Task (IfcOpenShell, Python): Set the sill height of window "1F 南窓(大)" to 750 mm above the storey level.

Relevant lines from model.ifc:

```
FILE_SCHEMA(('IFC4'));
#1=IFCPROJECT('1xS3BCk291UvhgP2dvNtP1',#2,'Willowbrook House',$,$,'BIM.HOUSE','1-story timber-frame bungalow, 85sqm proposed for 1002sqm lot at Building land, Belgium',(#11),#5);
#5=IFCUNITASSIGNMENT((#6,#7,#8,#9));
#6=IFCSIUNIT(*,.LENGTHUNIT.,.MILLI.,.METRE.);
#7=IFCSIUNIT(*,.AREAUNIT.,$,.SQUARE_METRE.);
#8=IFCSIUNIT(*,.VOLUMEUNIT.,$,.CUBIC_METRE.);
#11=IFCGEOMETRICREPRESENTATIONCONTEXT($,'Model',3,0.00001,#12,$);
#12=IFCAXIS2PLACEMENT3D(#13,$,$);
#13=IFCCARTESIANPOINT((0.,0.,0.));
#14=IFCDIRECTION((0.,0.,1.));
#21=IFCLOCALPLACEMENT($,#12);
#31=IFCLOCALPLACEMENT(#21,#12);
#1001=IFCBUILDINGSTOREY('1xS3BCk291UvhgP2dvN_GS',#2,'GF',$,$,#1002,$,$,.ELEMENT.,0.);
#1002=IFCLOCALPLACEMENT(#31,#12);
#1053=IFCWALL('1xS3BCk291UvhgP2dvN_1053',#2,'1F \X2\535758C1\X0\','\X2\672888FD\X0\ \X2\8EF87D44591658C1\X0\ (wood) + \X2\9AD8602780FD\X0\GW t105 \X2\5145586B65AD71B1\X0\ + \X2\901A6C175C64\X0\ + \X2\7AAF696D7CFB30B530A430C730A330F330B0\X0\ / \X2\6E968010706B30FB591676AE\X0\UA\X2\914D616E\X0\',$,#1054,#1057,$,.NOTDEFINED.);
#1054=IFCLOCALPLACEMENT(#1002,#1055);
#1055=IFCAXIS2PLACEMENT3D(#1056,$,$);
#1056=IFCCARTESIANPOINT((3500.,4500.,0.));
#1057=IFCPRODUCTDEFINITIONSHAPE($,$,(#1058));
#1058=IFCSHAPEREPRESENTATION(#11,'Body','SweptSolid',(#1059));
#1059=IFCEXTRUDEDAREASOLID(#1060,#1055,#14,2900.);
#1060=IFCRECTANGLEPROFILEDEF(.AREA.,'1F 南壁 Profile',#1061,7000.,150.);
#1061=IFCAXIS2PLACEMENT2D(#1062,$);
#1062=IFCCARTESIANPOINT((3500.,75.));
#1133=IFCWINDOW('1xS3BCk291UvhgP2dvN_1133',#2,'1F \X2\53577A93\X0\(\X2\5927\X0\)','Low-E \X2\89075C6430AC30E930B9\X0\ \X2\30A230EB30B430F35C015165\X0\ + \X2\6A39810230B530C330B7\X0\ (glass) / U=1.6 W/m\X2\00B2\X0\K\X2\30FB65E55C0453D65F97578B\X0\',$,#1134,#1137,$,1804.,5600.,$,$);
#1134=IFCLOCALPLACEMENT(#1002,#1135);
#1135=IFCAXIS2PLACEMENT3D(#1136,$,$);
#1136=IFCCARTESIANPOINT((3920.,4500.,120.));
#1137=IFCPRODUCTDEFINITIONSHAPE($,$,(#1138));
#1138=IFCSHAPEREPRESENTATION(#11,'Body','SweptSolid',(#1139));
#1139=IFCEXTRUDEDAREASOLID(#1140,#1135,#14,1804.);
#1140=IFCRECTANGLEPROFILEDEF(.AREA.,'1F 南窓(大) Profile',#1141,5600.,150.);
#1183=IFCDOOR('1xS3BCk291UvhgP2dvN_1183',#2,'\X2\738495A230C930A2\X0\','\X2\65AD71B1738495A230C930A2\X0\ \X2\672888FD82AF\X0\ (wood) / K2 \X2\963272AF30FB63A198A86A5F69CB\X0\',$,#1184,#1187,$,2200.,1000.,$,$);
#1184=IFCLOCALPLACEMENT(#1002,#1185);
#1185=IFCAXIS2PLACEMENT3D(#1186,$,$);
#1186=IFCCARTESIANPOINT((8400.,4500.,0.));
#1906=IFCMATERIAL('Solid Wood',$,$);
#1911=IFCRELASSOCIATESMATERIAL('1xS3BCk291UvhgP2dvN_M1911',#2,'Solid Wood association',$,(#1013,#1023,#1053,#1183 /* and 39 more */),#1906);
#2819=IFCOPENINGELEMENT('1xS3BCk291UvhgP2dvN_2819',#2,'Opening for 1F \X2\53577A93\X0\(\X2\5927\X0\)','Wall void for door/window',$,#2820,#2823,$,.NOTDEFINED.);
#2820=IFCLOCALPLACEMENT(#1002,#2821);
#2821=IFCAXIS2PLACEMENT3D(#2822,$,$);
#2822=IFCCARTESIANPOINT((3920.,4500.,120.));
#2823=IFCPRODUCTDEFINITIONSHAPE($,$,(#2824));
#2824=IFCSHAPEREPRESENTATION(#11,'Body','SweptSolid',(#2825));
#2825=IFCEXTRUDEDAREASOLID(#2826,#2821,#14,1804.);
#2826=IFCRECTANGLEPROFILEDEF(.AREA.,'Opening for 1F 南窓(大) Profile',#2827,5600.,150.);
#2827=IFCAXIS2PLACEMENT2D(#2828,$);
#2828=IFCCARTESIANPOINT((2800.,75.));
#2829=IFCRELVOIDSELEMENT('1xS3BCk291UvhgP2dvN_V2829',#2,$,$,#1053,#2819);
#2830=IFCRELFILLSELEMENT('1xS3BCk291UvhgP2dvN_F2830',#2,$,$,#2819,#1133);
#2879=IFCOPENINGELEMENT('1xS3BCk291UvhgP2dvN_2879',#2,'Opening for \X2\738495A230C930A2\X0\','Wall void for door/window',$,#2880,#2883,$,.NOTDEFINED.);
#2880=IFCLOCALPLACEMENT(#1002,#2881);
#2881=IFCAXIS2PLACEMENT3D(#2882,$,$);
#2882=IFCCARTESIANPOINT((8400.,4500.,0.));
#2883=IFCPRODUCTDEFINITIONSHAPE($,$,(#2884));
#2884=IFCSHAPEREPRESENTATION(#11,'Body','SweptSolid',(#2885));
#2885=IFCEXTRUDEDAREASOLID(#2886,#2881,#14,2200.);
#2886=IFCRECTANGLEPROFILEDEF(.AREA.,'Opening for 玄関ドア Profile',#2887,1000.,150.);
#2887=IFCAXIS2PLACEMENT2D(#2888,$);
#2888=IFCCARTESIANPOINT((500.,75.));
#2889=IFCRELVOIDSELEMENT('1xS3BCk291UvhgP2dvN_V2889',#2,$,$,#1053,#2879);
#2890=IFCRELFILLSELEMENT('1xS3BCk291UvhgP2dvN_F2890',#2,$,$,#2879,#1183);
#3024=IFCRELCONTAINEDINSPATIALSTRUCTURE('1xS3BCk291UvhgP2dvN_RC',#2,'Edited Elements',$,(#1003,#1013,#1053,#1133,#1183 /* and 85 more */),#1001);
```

```python
import numpy as np
import ifcopenshell
import ifcopenshell.api.geometry
import ifcopenshell.geom
import ifcopenshell.util.element
import ifcopenshell.util.placement
import ifcopenshell.util.shape
import ifcopenshell.util.unit

model = ifcopenshell.open("model.ifc")
unit_scale = ifcopenshell.util.unit.calculate_unit_scale(model)

window = model.by_id(1133)
opening = window.FillsVoids[0].RelatingOpeningElement
storey = ifcopenshell.util.element.get_container(window, ifc_class="IfcBuildingStorey")
level = ifcopenshell.util.placement.get_local_placement(storey.ObjectPlacement)[2, 3]

# The opening's origin need not be at the sill, so measure its lowest point.
shape = ifcopenshell.geom.create_shape(ifcopenshell.geom.settings(), opening)
bottom = ifcopenshell.util.shape.get_shape_bottom_elevation(shape, shape.geometry) / unit_scale
dz = level + 0.75 / unit_scale - bottom

shift = np.array([0.0, 0.0, dz])
# The window is not placed relative to its opening, so move both.
for product in (opening, window):
    matrix = ifcopenshell.util.placement.get_local_placement(product.ObjectPlacement)
    matrix[:3, 3] += shift
    ifcopenshell.api.geometry.edit_object_placement(model, product=product, matrix=matrix, is_si=False)

print(f"moved by {dz * unit_scale:+.3f} m")

model.write("model_rev.ifc")
```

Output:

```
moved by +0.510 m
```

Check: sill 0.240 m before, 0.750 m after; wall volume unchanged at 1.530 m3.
